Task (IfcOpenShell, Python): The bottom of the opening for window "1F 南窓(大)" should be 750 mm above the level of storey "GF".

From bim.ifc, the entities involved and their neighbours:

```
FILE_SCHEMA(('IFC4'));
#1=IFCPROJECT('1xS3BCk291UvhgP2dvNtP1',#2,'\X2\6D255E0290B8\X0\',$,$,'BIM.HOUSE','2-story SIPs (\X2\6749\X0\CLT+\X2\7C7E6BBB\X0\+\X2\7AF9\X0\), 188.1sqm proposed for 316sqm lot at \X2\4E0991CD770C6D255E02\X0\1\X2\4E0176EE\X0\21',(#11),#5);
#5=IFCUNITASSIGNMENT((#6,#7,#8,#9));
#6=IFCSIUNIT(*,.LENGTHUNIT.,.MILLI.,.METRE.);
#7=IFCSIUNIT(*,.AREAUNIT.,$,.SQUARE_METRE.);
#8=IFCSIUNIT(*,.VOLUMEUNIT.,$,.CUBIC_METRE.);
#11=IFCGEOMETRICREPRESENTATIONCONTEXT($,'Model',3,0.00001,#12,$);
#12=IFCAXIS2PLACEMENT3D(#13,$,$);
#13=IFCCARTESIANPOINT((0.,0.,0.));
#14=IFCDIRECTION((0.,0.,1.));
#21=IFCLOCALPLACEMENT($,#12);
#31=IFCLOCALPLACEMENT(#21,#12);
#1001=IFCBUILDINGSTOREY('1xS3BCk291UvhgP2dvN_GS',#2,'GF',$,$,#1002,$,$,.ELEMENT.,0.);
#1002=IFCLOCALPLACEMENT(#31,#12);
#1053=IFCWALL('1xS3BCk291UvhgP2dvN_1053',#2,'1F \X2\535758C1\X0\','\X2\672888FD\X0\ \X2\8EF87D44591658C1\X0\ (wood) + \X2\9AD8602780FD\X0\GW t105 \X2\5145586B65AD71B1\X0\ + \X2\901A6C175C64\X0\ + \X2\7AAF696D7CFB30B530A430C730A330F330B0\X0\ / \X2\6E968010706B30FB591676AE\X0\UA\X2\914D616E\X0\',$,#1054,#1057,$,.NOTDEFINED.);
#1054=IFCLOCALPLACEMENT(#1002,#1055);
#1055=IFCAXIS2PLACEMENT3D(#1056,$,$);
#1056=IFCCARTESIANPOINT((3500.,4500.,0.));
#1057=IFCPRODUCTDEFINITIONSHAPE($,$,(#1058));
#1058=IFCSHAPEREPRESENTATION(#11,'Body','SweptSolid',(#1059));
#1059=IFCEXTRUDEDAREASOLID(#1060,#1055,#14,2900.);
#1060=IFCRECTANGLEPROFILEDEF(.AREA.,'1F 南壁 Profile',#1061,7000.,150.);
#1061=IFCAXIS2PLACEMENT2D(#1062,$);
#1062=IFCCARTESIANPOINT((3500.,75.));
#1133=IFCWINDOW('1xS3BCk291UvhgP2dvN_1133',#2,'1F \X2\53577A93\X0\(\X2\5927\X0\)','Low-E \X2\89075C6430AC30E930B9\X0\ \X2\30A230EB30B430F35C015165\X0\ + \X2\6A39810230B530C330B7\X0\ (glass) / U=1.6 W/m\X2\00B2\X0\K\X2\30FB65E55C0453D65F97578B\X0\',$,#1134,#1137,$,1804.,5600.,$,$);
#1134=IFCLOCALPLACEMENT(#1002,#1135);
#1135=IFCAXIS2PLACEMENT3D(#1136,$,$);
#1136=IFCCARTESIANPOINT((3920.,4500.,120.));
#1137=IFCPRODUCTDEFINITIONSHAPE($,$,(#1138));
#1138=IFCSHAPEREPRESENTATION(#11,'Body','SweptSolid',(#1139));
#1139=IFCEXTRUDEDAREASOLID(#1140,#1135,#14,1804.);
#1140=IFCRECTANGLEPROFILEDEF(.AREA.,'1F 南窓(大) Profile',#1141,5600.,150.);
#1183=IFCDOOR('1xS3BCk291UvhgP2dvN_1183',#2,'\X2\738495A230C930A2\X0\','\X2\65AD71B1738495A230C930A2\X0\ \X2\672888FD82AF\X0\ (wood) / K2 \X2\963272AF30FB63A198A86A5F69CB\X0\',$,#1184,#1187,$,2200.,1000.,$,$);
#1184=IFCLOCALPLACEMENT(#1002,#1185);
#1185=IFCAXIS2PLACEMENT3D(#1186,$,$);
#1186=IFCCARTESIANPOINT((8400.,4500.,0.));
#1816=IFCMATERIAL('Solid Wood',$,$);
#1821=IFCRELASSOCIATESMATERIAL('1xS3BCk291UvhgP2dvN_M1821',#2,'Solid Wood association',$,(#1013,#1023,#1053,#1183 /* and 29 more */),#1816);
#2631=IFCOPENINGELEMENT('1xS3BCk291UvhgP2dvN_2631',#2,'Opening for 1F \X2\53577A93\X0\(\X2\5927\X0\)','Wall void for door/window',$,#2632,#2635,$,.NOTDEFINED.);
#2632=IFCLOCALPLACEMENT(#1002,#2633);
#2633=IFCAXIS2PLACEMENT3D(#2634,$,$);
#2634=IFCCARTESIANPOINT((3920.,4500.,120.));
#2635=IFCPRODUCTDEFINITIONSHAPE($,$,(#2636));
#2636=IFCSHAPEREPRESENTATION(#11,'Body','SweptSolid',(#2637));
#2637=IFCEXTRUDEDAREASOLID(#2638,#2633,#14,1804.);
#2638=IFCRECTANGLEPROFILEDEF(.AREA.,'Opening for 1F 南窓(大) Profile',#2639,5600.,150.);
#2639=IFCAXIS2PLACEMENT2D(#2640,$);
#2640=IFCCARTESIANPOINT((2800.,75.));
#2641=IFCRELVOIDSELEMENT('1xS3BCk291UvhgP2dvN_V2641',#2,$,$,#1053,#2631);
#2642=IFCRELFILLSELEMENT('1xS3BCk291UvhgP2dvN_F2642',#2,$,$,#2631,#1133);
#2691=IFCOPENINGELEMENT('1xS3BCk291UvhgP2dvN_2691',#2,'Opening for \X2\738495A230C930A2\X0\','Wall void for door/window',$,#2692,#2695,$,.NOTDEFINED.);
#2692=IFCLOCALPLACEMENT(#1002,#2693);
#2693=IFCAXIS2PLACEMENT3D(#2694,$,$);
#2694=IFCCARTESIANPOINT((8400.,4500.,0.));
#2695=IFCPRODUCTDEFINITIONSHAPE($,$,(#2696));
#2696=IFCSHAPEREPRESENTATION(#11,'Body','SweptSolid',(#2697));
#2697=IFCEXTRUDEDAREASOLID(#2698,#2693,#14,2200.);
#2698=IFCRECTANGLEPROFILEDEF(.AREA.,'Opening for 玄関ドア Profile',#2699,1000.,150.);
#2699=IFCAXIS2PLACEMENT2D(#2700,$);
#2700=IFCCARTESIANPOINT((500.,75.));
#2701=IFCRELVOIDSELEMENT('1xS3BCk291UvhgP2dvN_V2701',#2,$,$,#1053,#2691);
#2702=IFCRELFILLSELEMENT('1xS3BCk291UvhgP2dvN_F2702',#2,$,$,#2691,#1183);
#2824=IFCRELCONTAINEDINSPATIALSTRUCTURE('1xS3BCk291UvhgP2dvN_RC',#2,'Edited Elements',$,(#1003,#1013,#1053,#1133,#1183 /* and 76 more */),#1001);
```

```python
import numpy as np
import ifcopenshell
import ifcopenshell.api.geometry
import ifcopenshell.geom
import ifcopenshell.util.element
import ifcopenshell.util.placement
import ifcopenshell.util.shape
import ifcopenshell.util.unit

model = ifcopenshell.open("bim.ifc")
unit_scale = ifcopenshell.util.unit.calculate_unit_scale(model)

window = model.by_guid("1xS3BCk291UvhgP2dvN_1133")
opening = window.FillsVoids[0].RelatingOpeningElement
storey = ifcopenshell.util.element.get_container(window, ifc_class="IfcBuildingStorey")
level = ifcopenshell.util.placement.get_local_placement(storey.ObjectPlacement)[2, 3]

# The opening's origin need not be at the sill, so measure its lowest point.
shape = ifcopenshell.geom.create_shape(ifcopenshell.geom.settings(), opening)
bottom = ifcopenshell.util.shape.get_shape_bottom_elevation(shape, shape.geometry) / unit_scale
dz = level + 750.0 - bottom

shift = np.array([0.0, 0.0, dz])
# The window is not placed relative to its opening, so move both.
for product in (opening, window):
    matrix = ifcopenshell.util.placement.get_local_placement(product.ObjectPlacement)
    matrix[:3, 3] += shift
    ifcopenshell.api.geometry.edit_object_placement(model, product=product, matrix=matrix, is_si=False)

print(f"moved by {dz * unit_scale:+.3f} m")

model.write("bim-out.ifc")
```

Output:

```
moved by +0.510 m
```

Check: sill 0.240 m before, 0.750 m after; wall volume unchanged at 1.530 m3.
